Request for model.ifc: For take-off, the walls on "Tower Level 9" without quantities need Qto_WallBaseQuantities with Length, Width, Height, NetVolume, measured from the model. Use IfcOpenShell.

First a look at what the model holds.

```python
import ifcopenshell
import ifcopenshell.util.element
import ifcopenshell.util.unit

model = ifcopenshell.open("model.ifc")
print(model.schema)
for unit_type in ("LENGTHUNIT", "AREAUNIT", "VOLUMEUNIT"):
    print(unit_type, ifcopenshell.util.unit.calculate_unit_scale(model, unit_type))
storey = next(s for s in model.by_type("IfcBuildingStorey") if s.Name == "Tower Level 9")
walls = [e for e in ifcopenshell.util.element.get_decomposition(storey) if e.is_a("IfcWall")]
for e in sorted(walls, key=lambda e: e.id()):
    print(e.id(), e.is_a(), e.Name, list(ifcopenshell.util.element.get_psets(e, qtos_only=True)), sep=" | ")
```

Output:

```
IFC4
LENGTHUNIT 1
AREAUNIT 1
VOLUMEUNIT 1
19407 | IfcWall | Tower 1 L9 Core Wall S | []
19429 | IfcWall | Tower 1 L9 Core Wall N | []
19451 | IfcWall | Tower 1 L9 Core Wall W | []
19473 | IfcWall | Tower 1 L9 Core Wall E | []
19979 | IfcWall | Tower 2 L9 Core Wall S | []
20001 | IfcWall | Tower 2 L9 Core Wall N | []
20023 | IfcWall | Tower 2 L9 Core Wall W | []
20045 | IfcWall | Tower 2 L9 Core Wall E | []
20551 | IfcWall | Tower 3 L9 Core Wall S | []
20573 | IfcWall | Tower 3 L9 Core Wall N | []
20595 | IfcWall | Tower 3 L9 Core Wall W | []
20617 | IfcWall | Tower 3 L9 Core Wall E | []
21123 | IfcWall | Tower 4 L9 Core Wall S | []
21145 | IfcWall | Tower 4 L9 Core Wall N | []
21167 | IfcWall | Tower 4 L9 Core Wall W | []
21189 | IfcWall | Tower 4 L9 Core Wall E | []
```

```python
import ifcopenshell
import ifcopenshell.api.pset
import ifcopenshell.geom
import ifcopenshell.util.element
import ifcopenshell.util.shape
import ifcopenshell.util.unit

model = ifcopenshell.open("model.ifc")
unit_scale = ifcopenshell.util.unit.calculate_unit_scale(model)
volume_scale = ifcopenshell.util.unit.calculate_unit_scale(model, "VOLUMEUNIT")
settings = ifcopenshell.geom.settings()

storey = next(s for s in model.by_type("IfcBuildingStorey") if s.Name == "Tower Level 9")
walls = [e for e in ifcopenshell.util.element.get_decomposition(storey) if e.is_a("IfcWall")]

for e in sorted(walls, key=lambda e: e.id()):
    if ifcopenshell.util.element.get_psets(e, qtos_only=True, should_inherit=False):
        continue
    # Geometry comes back in metres, in the element's own axes.
    shape = ifcopenshell.geom.create_shape(settings, e)
    values = {
        "Length": ifcopenshell.util.shape.get_x(shape.geometry) / unit_scale,
        "Width": ifcopenshell.util.shape.get_y(shape.geometry) / unit_scale,
        "Height": ifcopenshell.util.shape.get_z(shape.geometry) / unit_scale,
        "NetVolume": ifcopenshell.util.shape.get_volume(shape.geometry) / volume_scale,
    }
    qto = ifcopenshell.api.pset.add_qto(model, product=e, name="Qto_WallBaseQuantities")
    ifcopenshell.api.pset.edit_qto(model, qto=qto, properties=values)
    print(e.id(), {k: round(v, 3) for k, v in values.items()})

model.write("model-out.ifc")
```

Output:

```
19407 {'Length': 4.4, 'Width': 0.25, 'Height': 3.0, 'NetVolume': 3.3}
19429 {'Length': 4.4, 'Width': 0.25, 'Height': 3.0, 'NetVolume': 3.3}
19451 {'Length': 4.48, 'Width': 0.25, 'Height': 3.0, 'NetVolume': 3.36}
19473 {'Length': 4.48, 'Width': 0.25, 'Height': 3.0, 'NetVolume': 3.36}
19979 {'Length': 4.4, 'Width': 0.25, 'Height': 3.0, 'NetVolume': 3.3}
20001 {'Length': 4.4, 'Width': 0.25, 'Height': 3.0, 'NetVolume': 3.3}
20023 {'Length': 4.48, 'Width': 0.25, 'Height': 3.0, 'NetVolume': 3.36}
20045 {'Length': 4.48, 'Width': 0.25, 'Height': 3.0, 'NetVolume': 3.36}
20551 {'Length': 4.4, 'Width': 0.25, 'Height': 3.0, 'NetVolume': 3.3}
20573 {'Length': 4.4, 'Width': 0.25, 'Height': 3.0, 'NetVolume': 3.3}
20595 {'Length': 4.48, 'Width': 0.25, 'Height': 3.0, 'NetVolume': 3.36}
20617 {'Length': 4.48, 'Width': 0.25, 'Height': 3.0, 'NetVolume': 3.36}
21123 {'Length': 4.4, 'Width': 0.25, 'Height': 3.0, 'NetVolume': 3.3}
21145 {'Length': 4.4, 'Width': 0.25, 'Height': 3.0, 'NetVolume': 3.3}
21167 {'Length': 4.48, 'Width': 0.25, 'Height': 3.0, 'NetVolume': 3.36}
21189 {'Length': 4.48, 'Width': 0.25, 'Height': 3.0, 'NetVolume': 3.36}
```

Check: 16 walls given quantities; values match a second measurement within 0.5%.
